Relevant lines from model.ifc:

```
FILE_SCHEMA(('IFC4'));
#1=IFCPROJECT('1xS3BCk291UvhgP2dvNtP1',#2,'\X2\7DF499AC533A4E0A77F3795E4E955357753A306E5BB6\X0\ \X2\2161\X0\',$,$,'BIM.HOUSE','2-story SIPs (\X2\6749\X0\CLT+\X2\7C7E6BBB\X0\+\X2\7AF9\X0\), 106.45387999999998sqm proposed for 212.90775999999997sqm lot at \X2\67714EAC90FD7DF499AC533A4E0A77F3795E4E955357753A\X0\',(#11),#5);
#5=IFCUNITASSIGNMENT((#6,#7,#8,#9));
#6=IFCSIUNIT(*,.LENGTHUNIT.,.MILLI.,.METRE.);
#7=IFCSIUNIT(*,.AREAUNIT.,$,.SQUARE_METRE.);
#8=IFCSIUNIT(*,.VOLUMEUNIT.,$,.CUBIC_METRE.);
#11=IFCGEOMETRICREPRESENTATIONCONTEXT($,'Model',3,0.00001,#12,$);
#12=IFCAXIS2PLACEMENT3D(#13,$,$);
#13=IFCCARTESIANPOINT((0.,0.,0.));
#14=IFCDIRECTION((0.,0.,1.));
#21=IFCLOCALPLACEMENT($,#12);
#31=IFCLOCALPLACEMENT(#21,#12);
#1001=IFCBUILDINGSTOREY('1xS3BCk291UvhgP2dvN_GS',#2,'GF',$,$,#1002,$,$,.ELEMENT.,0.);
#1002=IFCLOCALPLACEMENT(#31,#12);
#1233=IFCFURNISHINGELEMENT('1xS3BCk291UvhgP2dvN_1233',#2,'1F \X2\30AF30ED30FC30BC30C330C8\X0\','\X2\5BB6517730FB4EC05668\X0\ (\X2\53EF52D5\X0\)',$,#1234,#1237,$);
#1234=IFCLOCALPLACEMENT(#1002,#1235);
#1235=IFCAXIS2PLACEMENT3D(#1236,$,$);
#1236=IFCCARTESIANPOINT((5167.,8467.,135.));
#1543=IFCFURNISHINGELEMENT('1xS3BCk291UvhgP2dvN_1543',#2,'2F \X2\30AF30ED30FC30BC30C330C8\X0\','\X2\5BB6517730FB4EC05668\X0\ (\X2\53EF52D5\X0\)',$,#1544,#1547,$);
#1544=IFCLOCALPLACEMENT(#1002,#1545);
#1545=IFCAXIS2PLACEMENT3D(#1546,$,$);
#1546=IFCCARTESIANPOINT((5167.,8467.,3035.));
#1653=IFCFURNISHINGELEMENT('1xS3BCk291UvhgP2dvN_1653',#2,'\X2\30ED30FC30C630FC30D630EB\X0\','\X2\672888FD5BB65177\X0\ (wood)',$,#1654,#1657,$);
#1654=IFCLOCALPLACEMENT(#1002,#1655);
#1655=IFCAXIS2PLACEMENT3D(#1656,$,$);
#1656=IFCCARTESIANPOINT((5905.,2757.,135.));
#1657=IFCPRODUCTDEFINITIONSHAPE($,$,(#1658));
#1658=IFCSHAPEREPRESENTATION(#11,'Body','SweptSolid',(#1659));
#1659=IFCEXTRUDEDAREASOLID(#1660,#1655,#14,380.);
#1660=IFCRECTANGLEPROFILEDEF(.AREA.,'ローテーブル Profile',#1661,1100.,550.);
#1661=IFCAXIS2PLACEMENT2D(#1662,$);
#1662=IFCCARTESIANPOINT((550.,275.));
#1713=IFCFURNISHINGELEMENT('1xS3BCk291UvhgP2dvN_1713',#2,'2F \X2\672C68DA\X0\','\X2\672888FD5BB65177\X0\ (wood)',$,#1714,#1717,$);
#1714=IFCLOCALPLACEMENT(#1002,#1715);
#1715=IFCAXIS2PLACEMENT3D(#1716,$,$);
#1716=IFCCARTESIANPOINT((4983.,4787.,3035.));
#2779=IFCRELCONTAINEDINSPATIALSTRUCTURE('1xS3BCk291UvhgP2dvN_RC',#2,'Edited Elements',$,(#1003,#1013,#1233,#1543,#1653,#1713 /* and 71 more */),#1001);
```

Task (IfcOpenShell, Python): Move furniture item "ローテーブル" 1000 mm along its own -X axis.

```python
import ifcopenshell
import ifcopenshell.api.geometry
import ifcopenshell.util.placement

model = ifcopenshell.open("model.ifc")

item = model.by_id(1653)
matrix = ifcopenshell.util.placement.get_local_placement(item.ObjectPlacement)
matrix[:3, 3] -= matrix[:3, 0] * 1000.0
ifcopenshell.api.geometry.edit_object_placement(model, product=item, matrix=matrix, is_si=False)

print(ifcopenshell.util.placement.get_local_placement(item.ObjectPlacement).round(3) + 0.0)

model.write("model_edited.ifc")
```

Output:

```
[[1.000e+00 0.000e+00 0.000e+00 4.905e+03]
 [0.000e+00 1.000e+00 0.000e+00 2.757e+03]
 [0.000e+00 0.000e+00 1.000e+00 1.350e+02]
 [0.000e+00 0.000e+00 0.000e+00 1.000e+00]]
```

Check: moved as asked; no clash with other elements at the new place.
